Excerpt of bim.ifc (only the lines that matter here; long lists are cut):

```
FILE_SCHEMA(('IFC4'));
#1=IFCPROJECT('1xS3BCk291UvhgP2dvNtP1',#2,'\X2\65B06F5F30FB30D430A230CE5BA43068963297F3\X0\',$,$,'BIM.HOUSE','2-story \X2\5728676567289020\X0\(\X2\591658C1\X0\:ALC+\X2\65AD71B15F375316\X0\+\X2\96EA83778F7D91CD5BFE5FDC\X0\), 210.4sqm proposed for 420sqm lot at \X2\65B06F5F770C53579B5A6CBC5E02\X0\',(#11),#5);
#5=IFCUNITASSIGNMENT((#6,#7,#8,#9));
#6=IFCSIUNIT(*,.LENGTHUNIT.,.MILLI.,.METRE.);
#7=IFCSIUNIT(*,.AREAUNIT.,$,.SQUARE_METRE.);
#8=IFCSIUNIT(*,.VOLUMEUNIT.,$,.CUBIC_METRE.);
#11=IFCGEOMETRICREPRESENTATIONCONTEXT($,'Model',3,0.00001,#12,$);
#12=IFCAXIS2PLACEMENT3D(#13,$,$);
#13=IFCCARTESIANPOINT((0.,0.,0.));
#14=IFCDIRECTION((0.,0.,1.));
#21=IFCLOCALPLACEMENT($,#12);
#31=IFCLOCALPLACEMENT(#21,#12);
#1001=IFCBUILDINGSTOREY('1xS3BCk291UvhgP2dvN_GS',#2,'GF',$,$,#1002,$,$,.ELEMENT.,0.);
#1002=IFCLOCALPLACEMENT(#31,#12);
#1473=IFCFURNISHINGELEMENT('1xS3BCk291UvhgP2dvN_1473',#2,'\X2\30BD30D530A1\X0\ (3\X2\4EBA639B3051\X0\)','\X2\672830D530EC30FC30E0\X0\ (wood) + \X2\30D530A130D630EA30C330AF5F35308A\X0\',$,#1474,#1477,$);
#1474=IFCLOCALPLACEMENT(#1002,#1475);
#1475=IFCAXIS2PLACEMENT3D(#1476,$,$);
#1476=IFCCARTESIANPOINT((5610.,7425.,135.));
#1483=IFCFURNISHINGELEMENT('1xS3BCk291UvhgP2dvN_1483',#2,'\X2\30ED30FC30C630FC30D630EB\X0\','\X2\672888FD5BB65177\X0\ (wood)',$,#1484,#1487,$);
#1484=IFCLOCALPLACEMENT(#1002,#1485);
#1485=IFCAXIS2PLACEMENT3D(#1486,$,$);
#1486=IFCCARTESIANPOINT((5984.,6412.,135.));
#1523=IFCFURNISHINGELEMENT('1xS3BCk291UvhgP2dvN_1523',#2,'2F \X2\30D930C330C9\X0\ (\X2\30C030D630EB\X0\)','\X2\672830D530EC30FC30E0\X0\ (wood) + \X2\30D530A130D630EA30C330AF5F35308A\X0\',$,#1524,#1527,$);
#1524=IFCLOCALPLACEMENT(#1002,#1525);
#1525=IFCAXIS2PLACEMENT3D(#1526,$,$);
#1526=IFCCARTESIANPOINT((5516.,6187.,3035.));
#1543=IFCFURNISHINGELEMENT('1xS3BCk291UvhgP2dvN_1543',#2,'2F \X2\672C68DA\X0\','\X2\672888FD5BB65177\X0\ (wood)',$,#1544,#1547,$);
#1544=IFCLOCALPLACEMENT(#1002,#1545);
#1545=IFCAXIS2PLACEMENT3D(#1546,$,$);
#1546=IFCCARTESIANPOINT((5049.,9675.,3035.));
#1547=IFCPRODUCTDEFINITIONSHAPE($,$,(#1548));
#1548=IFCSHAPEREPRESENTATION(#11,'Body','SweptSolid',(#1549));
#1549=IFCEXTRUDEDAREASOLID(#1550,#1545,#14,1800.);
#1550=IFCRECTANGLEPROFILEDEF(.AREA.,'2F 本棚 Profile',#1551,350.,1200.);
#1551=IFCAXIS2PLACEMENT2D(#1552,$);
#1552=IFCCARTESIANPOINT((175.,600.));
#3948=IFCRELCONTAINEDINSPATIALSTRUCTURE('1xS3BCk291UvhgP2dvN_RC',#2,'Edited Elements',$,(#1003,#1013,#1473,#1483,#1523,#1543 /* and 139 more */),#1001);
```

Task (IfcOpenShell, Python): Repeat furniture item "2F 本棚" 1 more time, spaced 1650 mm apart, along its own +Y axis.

```python
import ifcopenshell
import ifcopenshell.api.geometry
import ifcopenshell.api.root
import ifcopenshell.util.element
import ifcopenshell.util.placement
import ifcopenshell.util.unit

model = ifcopenshell.open("bim.ifc")
unit_scale = ifcopenshell.util.unit.calculate_unit_scale(model)


def reuse_history(source, copy):
    """copy_class also copies each property set's owner history, people and application; keep the originals."""
    for rel in copy.IsDefinedBy:
        if rel.is_a("IfcRelDefinesByProperties") and (history := rel.RelatingPropertyDefinition.OwnerHistory):
            rel.RelatingPropertyDefinition.OwnerHistory = source.OwnerHistory
            ifcopenshell.util.element.remove_deep2(model, history)


source = model.by_id(1543)
base = ifcopenshell.util.placement.get_local_placement(source.ObjectPlacement)
step = base[:3, 1] * 1.65 / unit_scale

for i in range(1, 2):
    copy = ifcopenshell.api.root.copy_class(model, product=source)
    copy.Representation = ifcopenshell.util.element.copy_deep(
        model, source.Representation, exclude=["IfcGeometricRepresentationContext", "IfcRepresentationMap"]
    )
    reuse_history(source, copy)
    matrix = base.copy()
    matrix[:3, 3] += i * step
    print("added at", matrix[:3, 3].round(3) + 0.0)
    ifcopenshell.api.geometry.edit_object_placement(model, product=copy, matrix=matrix, is_si=False)

model.write("bim_edited.ifc")
```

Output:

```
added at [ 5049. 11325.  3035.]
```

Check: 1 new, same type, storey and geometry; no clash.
